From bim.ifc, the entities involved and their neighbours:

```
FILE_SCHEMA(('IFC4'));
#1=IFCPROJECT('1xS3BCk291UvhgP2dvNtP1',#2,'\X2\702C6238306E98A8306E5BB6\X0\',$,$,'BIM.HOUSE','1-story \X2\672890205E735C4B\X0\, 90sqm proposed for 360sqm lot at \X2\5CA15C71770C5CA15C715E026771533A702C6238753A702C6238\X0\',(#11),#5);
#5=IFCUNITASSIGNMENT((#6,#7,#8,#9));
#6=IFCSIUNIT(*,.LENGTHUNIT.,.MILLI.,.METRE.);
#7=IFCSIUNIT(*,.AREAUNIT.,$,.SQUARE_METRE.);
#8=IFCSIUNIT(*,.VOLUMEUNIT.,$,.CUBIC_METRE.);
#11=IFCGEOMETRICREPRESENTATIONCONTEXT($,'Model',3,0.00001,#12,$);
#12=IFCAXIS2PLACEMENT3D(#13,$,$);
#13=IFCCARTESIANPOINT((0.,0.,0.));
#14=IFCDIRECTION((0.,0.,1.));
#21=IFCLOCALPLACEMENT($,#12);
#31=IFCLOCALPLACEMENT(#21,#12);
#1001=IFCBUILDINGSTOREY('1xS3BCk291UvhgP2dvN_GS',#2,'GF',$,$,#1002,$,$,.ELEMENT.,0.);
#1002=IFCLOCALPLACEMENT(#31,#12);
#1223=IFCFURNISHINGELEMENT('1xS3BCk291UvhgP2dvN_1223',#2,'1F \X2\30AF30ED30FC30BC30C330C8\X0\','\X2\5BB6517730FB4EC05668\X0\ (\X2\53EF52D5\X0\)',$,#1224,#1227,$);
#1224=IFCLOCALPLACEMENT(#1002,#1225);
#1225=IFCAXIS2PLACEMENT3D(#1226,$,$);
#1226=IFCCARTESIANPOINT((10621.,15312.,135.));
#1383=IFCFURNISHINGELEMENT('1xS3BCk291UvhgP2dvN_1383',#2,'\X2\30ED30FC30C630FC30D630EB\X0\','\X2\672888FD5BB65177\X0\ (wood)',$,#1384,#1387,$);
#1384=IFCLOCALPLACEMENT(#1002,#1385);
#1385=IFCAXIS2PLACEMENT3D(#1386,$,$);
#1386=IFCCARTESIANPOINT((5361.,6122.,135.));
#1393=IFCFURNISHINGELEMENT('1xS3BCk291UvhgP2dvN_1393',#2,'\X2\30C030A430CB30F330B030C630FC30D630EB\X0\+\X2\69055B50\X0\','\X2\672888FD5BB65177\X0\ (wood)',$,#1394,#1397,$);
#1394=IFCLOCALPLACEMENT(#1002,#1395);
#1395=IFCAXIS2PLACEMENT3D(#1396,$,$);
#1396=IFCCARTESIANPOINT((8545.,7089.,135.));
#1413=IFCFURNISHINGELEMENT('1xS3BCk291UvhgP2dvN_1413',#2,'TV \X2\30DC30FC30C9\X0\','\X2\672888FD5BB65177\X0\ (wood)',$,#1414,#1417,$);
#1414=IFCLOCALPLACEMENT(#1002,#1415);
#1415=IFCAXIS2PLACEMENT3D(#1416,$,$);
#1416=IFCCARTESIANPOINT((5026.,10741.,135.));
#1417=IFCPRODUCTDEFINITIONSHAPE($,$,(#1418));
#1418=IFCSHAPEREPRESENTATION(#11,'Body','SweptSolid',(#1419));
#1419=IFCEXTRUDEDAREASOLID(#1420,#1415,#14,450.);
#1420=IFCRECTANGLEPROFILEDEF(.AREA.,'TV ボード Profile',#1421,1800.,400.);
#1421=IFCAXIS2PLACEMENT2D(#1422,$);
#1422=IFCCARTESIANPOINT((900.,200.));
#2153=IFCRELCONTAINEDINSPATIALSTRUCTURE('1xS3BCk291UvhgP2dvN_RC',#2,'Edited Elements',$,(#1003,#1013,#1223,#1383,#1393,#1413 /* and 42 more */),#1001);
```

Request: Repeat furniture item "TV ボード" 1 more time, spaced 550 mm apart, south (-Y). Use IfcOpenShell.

```python
import numpy as np
import ifcopenshell
import ifcopenshell.api.geometry
import ifcopenshell.api.root
import ifcopenshell.util.element
import ifcopenshell.util.placement
import ifcopenshell.util.unit

model = ifcopenshell.open("bim.ifc")
unit_scale = ifcopenshell.util.unit.calculate_unit_scale(model)


def reuse_history(source, copy):
    """copy_class also copies each property set's owner history, people and application; keep the originals."""
    for rel in copy.IsDefinedBy:
        if rel.is_a("IfcRelDefinesByProperties") and (history := rel.RelatingPropertyDefinition.OwnerHistory):
            rel.RelatingPropertyDefinition.OwnerHistory = source.OwnerHistory
            ifcopenshell.util.element.remove_deep2(model, history)


source = model.by_guid("1xS3BCk291UvhgP2dvN_1413")
base = ifcopenshell.util.placement.get_local_placement(source.ObjectPlacement)
step = np.array([0.0, -1.0, 0.0]) * 0.55 / unit_scale

for i in range(1, 2):
    copy = ifcopenshell.api.root.copy_class(model, product=source)
    copy.Representation = ifcopenshell.util.element.copy_deep(
        model, source.Representation, exclude=["IfcGeometricRepresentationContext", "IfcRepresentationMap"]
    )
    reuse_history(source, copy)
    matrix = base.copy()
    matrix[:3, 3] += i * step
    print("added at", matrix[:3, 3].round(3) + 0.0)
    ifcopenshell.api.geometry.edit_object_placement(model, product=copy, matrix=matrix, is_si=False)

model.write("bim_v2.ifc")
```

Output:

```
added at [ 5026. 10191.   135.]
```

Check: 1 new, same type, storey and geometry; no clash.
